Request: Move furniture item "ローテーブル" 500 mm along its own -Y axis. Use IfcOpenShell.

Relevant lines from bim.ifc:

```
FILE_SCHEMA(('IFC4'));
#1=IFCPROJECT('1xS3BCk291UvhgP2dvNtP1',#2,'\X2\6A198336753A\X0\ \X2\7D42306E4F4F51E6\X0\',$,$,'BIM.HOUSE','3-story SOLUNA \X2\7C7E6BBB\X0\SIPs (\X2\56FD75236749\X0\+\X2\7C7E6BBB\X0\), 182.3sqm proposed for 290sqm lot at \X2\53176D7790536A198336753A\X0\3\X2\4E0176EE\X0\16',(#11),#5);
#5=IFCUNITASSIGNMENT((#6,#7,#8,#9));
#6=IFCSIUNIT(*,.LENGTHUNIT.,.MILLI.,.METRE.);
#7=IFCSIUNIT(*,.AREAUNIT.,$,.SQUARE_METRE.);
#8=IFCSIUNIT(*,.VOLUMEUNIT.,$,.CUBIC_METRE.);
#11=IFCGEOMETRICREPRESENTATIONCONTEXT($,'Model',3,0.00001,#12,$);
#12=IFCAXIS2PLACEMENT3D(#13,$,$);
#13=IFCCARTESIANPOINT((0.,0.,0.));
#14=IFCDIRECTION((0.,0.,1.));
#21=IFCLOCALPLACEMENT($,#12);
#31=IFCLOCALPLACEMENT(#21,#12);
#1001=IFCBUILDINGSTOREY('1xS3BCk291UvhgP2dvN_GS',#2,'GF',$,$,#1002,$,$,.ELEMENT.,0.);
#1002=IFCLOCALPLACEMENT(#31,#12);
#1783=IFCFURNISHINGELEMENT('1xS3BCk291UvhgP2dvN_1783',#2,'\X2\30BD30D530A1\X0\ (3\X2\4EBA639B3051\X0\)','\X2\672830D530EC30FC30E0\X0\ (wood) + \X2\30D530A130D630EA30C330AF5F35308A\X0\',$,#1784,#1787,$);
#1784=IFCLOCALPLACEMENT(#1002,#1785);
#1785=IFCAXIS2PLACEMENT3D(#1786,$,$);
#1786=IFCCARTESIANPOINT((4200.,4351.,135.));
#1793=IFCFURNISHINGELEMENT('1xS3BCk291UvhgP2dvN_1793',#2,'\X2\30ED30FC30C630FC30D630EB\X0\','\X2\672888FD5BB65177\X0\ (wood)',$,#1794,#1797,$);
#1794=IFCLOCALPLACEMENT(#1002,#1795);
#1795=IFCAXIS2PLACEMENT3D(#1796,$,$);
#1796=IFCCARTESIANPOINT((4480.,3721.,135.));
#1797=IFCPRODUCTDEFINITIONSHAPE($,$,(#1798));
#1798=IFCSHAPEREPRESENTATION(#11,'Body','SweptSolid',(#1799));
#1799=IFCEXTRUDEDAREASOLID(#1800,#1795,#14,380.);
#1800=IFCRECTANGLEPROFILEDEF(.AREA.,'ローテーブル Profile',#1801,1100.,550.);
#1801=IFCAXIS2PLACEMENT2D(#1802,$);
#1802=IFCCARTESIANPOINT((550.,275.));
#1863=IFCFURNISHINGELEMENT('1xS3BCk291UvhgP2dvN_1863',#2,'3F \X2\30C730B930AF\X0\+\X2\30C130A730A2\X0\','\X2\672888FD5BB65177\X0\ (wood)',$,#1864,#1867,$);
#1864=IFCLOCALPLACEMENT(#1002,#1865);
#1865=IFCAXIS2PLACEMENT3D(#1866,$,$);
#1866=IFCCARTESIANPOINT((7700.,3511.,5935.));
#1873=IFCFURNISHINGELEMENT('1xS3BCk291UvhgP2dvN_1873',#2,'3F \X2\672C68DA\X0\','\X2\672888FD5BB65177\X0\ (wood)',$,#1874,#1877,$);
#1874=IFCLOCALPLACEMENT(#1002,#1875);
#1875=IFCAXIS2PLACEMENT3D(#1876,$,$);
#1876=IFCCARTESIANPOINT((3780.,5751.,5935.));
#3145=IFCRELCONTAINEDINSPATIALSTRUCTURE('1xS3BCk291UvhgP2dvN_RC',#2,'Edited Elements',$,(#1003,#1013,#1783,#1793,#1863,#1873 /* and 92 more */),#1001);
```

```python
import ifcopenshell
import ifcopenshell.api.geometry
import ifcopenshell.util.placement
import ifcopenshell.util.unit

model = ifcopenshell.open("bim.ifc")
unit_scale = ifcopenshell.util.unit.calculate_unit_scale(model)

item = model.by_guid("1xS3BCk291UvhgP2dvN_1793")
matrix = ifcopenshell.util.placement.get_local_placement(item.ObjectPlacement)
matrix[:3, 3] -= matrix[:3, 1] * 0.5 / unit_scale
ifcopenshell.api.geometry.edit_object_placement(model, product=item, matrix=matrix, is_si=False)

print(ifcopenshell.util.placement.get_local_placement(item.ObjectPlacement).round(3) + 0.0)

model.write("bim_updated.ifc")
```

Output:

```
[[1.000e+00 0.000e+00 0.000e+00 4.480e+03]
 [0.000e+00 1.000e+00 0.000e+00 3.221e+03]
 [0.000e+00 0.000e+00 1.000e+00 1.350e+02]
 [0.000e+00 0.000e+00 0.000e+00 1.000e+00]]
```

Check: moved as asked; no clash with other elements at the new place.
